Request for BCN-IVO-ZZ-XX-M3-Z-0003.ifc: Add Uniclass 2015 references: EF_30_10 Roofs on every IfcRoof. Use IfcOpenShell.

First a look at what the model holds.

```python
import ifcopenshell

model = ifcopenshell.open("BCN-IVO-ZZ-XX-M3-Z-0003.ifc")
print(model.schema)
print("classifications:", [c.Name for c in model.by_type("IfcClassification")])
for ifc_class in ("IfcDoor", "IfcRoof", "IfcStair", "IfcWall", "IfcWindow"):
    print(ifc_class, len(model.by_type(ifc_class)))
```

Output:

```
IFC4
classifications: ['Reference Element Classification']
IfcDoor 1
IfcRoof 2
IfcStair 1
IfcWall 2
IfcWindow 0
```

```python
import ifcopenshell
import ifcopenshell.api.classification

model = ifcopenshell.open("BCN-IVO-ZZ-XX-M3-Z-0003.ifc")

system = ifcopenshell.api.classification.add_classification(model, classification="Uniclass 2015")

codes = {
    "IfcRoof": ("EF_30_10", "Roofs"),
}
for ifc_class, (code, name) in codes.items():
    products = model.by_type(ifc_class)
    ifcopenshell.api.classification.add_reference(
        model, products=products, classification=system, identification=code, name=name
    )
    print(code, len(products))

model.write("BCN-IVO-ZZ-XX-M3-Z-0003_edited.ifc")
```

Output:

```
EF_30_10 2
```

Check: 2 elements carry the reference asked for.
